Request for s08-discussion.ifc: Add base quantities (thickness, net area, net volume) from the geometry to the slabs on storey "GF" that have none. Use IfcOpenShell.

First a look at what the model holds.

```python
import ifcopenshell
import ifcopenshell.util.element
import ifcopenshell.util.unit

model = ifcopenshell.open("s08-discussion.ifc")
print(model.schema)
for unit_type in ("LENGTHUNIT", "AREAUNIT", "VOLUMEUNIT"):
    print(unit_type, ifcopenshell.util.unit.calculate_unit_scale(model, unit_type))
storey = next(s for s in model.by_type("IfcBuildingStorey") if s.Name == "GF")
slabs = [e for e in ifcopenshell.util.element.get_decomposition(storey) if e.is_a("IfcSlab")]
for e in sorted(slabs, key=lambda e: e.id()):
    print(e.id(), e.is_a(), e.Name, list(ifcopenshell.util.element.get_psets(e, qtos_only=True)), sep=" | ")
```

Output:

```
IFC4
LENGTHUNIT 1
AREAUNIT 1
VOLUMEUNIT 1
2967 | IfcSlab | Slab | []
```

```python
import ifcopenshell
import ifcopenshell.api.pset
import ifcopenshell.geom
import ifcopenshell.util.element
import ifcopenshell.util.shape
import ifcopenshell.util.unit

model = ifcopenshell.open("s08-discussion.ifc")
unit_scale = ifcopenshell.util.unit.calculate_unit_scale(model)
area_scale = ifcopenshell.util.unit.calculate_unit_scale(model, "AREAUNIT")
volume_scale = ifcopenshell.util.unit.calculate_unit_scale(model, "VOLUMEUNIT")
settings = ifcopenshell.geom.settings()

storey = next(s for s in model.by_type("IfcBuildingStorey") if s.Name == "GF")
slabs = [e for e in ifcopenshell.util.element.get_decomposition(storey) if e.is_a("IfcSlab")]

for e in sorted(slabs, key=lambda e: e.id()):
    if ifcopenshell.util.element.get_psets(e, qtos_only=True, should_inherit=False):
        continue
    # Geometry comes back in metres, in the element's own axes.
    shape = ifcopenshell.geom.create_shape(settings, e)
    values = {
        "Width": ifcopenshell.util.shape.get_z(shape.geometry) / unit_scale,
        "NetArea": ifcopenshell.util.shape.get_footprint_area(shape.geometry) / area_scale,
        "NetVolume": ifcopenshell.util.shape.get_volume(shape.geometry) / volume_scale,
    }
    qto = ifcopenshell.api.pset.add_qto(model, product=e, name="Qto_SlabBaseQuantities")
    ifcopenshell.api.pset.edit_qto(model, qto=qto, properties=values)
    print(e.id(), {k: round(v, 3) for k, v in values.items()})

model.write("s08-discussion_updated.ifc")
```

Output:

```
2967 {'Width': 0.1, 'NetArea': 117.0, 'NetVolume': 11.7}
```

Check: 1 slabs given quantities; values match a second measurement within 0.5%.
